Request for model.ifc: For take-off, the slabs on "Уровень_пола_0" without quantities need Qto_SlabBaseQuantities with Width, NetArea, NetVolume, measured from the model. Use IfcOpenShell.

First a look at what the model holds.

```python
import ifcopenshell
import ifcopenshell.util.element
import ifcopenshell.util.unit

model = ifcopenshell.open("model.ifc")
print(model.schema)
for unit_type in ("LENGTHUNIT", "AREAUNIT", "VOLUMEUNIT"):
    print(unit_type, ifcopenshell.util.unit.calculate_unit_scale(model, unit_type))
storey = next(s for s in model.by_type("IfcBuildingStorey") if s.Name == "Уровень_пола_0")
slabs = [e for e in ifcopenshell.util.element.get_decomposition(storey) if e.is_a("IfcSlab")]
for e in sorted(slabs, key=lambda e: e.id()):
    print(e.id(), e.is_a(), e.Name, list(ifcopenshell.util.element.get_psets(e, qtos_only=True)), sep=" | ")
```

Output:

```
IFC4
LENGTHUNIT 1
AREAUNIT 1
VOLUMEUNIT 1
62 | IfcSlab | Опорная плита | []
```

```python
import ifcopenshell
import ifcopenshell.api.pset
import ifcopenshell.geom
import ifcopenshell.util.element
import ifcopenshell.util.shape
import ifcopenshell.util.unit

model = ifcopenshell.open("model.ifc")
unit_scale = ifcopenshell.util.unit.calculate_unit_scale(model)
area_scale = ifcopenshell.util.unit.calculate_unit_scale(model, "AREAUNIT")
volume_scale = ifcopenshell.util.unit.calculate_unit_scale(model, "VOLUMEUNIT")
settings = ifcopenshell.geom.settings()

storey = next(s for s in model.by_type("IfcBuildingStorey") if s.Name == "Уровень_пола_0")
slabs = [e for e in ifcopenshell.util.element.get_decomposition(storey) if e.is_a("IfcSlab")]

for e in sorted(slabs, key=lambda e: e.id()):
    if ifcopenshell.util.element.get_psets(e, qtos_only=True, should_inherit=False):
        continue
    # Geometry comes back in metres, in the element's own axes.
    shape = ifcopenshell.geom.create_shape(settings, e)
    values = {
        "Width": ifcopenshell.util.shape.get_z(shape.geometry) / unit_scale,
        "NetArea": ifcopenshell.util.shape.get_footprint_area(shape.geometry) / area_scale,
        "NetVolume": ifcopenshell.util.shape.get_volume(shape.geometry) / volume_scale,
    }
    qto = ifcopenshell.api.pset.add_qto(model, product=e, name="Qto_SlabBaseQuantities")
    ifcopenshell.api.pset.edit_qto(model, qto=qto, properties=values)
    print(e.id(), {k: round(v, 3) for k, v in values.items()})

model.write("model_updated.ifc")
```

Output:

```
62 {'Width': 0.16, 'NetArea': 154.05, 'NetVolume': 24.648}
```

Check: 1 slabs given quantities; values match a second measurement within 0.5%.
